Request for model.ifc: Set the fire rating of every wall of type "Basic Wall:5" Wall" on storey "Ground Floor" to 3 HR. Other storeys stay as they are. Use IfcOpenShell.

First a look at what the model holds.

```python
import ifcopenshell
import ifcopenshell.util.element

model = ifcopenshell.open("model.ifc")
print(model.schema)
storey = next(s for s in model.by_type("IfcBuildingStorey") if s.Name == "Ground Floor")
walls = [e for e in ifcopenshell.util.element.get_decomposition(storey) if e.is_a("IfcWall")]
seen = {}
for e in walls:
    element_type = ifcopenshell.util.element.get_type(e)
    key = (element_type.Name if element_type != e and element_type else None, ifcopenshell.util.element.get_pset(e, "Pset_WallCommon", "FireRating"))
    seen[key] = seen.get(key, 0) + 1
for (name, value), count in sorted(seen.items(), key=str):
    print(count, "x", name, "|", value)
```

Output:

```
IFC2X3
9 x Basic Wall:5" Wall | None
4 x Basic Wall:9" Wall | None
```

```python
import ifcopenshell
import ifcopenshell.api.pset
import ifcopenshell.util.element

model = ifcopenshell.open("model.ifc")

storey = next(s for s in model.by_type("IfcBuildingStorey") if s.Name == "Ground Floor")
walls = [e for e in ifcopenshell.util.element.get_decomposition(storey) if e.is_a("IfcWall")]

count = 0
for e in walls:
    element_type = ifcopenshell.util.element.get_type(e)
    if element_type in (None, e) or element_type.Name != 'Basic Wall:5" Wall':
        continue
    # add_pset returns the element's existing set when there is one.
    pset = ifcopenshell.api.pset.add_pset(model, product=e, name="Pset_WallCommon")
    ifcopenshell.api.pset.edit_pset(model, pset=pset, properties={"FireRating": "3 HR"})
    count += 1

print(count, "walls updated")

model.write("model_v2.ifc")
```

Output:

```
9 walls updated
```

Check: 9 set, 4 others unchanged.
